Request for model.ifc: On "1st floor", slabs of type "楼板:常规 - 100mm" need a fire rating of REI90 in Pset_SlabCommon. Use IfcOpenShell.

First a look at what the model holds.

```python
import ifcopenshell
import ifcopenshell.util.element

model = ifcopenshell.open("model.ifc")
print(model.schema)
storey = next(s for s in model.by_type("IfcBuildingStorey") if s.Name == "1st floor")
slabs = [e for e in ifcopenshell.util.element.get_decomposition(storey) if e.is_a("IfcSlab")]
seen = {}
for e in slabs:
    element_type = ifcopenshell.util.element.get_type(e)
    key = (element_type.Name if element_type != e and element_type else None, ifcopenshell.util.element.get_pset(e, "Pset_SlabCommon", "FireRating"))
    seen[key] = seen.get(key, 0) + 1
for (name, value), count in sorted(seen.items(), key=str):
    print(count, "x", name, "|", value)
```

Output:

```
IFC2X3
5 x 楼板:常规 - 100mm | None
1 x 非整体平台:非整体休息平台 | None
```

```python
import ifcopenshell
import ifcopenshell.api.pset
import ifcopenshell.util.element

model = ifcopenshell.open("model.ifc")

storey = next(s for s in model.by_type("IfcBuildingStorey") if s.Name == "1st floor")
slabs = [e for e in ifcopenshell.util.element.get_decomposition(storey) if e.is_a("IfcSlab")]

count = 0
for e in slabs:
    element_type = ifcopenshell.util.element.get_type(e)
    if element_type in (None, e) or element_type.Name != "楼板:常规 - 100mm":
        continue
    # add_pset returns the element's existing set when there is one.
    pset = ifcopenshell.api.pset.add_pset(model, product=e, name="Pset_SlabCommon")
    ifcopenshell.api.pset.edit_pset(model, pset=pset, properties={"FireRating": "REI90"})
    count += 1

print(count, "slabs updated")

model.write("model_rev.ifc")
```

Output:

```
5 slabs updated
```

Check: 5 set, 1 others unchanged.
